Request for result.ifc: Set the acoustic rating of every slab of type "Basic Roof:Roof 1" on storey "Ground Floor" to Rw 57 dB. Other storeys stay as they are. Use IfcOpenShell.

First a look at what the model holds.

```python
import ifcopenshell
import ifcopenshell.util.element

model = ifcopenshell.open("result.ifc")
print(model.schema)
storey = next(s for s in model.by_type("IfcBuildingStorey") if s.Name == "Ground Floor")
slabs = [e for e in ifcopenshell.util.element.get_decomposition(storey) if e.is_a("IfcSlab")]
seen = {}
for e in slabs:
    element_type = ifcopenshell.util.element.get_type(e)
    key = (element_type.Name if element_type != e and element_type else None, ifcopenshell.util.element.get_pset(e, "Pset_SlabCommon", "AcousticRating"))
    seen[key] = seen.get(key, 0) + 1
for (name, value), count in sorted(seen.items(), key=str):
    print(count, "x", name, "|", value)
```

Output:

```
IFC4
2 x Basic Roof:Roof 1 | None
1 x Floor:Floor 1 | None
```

```python
import ifcopenshell
import ifcopenshell.api.pset
import ifcopenshell.util.element

model = ifcopenshell.open("result.ifc")

storey = next(s for s in model.by_type("IfcBuildingStorey") if s.Name == "Ground Floor")
slabs = [e for e in ifcopenshell.util.element.get_decomposition(storey) if e.is_a("IfcSlab")]

count = 0
for e in slabs:
    element_type = ifcopenshell.util.element.get_type(e)
    if element_type in (None, e) or element_type.Name != "Basic Roof:Roof 1":
        continue
    # add_pset returns the element's existing set when there is one.
    pset = ifcopenshell.api.pset.add_pset(model, product=e, name="Pset_SlabCommon")
    ifcopenshell.api.pset.edit_pset(model, pset=pset, properties={"AcousticRating": "Rw 57 dB"})
    count += 1

print(count, "slabs updated")

model.write("result_edited.ifc")
```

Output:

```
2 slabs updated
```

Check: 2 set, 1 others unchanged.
